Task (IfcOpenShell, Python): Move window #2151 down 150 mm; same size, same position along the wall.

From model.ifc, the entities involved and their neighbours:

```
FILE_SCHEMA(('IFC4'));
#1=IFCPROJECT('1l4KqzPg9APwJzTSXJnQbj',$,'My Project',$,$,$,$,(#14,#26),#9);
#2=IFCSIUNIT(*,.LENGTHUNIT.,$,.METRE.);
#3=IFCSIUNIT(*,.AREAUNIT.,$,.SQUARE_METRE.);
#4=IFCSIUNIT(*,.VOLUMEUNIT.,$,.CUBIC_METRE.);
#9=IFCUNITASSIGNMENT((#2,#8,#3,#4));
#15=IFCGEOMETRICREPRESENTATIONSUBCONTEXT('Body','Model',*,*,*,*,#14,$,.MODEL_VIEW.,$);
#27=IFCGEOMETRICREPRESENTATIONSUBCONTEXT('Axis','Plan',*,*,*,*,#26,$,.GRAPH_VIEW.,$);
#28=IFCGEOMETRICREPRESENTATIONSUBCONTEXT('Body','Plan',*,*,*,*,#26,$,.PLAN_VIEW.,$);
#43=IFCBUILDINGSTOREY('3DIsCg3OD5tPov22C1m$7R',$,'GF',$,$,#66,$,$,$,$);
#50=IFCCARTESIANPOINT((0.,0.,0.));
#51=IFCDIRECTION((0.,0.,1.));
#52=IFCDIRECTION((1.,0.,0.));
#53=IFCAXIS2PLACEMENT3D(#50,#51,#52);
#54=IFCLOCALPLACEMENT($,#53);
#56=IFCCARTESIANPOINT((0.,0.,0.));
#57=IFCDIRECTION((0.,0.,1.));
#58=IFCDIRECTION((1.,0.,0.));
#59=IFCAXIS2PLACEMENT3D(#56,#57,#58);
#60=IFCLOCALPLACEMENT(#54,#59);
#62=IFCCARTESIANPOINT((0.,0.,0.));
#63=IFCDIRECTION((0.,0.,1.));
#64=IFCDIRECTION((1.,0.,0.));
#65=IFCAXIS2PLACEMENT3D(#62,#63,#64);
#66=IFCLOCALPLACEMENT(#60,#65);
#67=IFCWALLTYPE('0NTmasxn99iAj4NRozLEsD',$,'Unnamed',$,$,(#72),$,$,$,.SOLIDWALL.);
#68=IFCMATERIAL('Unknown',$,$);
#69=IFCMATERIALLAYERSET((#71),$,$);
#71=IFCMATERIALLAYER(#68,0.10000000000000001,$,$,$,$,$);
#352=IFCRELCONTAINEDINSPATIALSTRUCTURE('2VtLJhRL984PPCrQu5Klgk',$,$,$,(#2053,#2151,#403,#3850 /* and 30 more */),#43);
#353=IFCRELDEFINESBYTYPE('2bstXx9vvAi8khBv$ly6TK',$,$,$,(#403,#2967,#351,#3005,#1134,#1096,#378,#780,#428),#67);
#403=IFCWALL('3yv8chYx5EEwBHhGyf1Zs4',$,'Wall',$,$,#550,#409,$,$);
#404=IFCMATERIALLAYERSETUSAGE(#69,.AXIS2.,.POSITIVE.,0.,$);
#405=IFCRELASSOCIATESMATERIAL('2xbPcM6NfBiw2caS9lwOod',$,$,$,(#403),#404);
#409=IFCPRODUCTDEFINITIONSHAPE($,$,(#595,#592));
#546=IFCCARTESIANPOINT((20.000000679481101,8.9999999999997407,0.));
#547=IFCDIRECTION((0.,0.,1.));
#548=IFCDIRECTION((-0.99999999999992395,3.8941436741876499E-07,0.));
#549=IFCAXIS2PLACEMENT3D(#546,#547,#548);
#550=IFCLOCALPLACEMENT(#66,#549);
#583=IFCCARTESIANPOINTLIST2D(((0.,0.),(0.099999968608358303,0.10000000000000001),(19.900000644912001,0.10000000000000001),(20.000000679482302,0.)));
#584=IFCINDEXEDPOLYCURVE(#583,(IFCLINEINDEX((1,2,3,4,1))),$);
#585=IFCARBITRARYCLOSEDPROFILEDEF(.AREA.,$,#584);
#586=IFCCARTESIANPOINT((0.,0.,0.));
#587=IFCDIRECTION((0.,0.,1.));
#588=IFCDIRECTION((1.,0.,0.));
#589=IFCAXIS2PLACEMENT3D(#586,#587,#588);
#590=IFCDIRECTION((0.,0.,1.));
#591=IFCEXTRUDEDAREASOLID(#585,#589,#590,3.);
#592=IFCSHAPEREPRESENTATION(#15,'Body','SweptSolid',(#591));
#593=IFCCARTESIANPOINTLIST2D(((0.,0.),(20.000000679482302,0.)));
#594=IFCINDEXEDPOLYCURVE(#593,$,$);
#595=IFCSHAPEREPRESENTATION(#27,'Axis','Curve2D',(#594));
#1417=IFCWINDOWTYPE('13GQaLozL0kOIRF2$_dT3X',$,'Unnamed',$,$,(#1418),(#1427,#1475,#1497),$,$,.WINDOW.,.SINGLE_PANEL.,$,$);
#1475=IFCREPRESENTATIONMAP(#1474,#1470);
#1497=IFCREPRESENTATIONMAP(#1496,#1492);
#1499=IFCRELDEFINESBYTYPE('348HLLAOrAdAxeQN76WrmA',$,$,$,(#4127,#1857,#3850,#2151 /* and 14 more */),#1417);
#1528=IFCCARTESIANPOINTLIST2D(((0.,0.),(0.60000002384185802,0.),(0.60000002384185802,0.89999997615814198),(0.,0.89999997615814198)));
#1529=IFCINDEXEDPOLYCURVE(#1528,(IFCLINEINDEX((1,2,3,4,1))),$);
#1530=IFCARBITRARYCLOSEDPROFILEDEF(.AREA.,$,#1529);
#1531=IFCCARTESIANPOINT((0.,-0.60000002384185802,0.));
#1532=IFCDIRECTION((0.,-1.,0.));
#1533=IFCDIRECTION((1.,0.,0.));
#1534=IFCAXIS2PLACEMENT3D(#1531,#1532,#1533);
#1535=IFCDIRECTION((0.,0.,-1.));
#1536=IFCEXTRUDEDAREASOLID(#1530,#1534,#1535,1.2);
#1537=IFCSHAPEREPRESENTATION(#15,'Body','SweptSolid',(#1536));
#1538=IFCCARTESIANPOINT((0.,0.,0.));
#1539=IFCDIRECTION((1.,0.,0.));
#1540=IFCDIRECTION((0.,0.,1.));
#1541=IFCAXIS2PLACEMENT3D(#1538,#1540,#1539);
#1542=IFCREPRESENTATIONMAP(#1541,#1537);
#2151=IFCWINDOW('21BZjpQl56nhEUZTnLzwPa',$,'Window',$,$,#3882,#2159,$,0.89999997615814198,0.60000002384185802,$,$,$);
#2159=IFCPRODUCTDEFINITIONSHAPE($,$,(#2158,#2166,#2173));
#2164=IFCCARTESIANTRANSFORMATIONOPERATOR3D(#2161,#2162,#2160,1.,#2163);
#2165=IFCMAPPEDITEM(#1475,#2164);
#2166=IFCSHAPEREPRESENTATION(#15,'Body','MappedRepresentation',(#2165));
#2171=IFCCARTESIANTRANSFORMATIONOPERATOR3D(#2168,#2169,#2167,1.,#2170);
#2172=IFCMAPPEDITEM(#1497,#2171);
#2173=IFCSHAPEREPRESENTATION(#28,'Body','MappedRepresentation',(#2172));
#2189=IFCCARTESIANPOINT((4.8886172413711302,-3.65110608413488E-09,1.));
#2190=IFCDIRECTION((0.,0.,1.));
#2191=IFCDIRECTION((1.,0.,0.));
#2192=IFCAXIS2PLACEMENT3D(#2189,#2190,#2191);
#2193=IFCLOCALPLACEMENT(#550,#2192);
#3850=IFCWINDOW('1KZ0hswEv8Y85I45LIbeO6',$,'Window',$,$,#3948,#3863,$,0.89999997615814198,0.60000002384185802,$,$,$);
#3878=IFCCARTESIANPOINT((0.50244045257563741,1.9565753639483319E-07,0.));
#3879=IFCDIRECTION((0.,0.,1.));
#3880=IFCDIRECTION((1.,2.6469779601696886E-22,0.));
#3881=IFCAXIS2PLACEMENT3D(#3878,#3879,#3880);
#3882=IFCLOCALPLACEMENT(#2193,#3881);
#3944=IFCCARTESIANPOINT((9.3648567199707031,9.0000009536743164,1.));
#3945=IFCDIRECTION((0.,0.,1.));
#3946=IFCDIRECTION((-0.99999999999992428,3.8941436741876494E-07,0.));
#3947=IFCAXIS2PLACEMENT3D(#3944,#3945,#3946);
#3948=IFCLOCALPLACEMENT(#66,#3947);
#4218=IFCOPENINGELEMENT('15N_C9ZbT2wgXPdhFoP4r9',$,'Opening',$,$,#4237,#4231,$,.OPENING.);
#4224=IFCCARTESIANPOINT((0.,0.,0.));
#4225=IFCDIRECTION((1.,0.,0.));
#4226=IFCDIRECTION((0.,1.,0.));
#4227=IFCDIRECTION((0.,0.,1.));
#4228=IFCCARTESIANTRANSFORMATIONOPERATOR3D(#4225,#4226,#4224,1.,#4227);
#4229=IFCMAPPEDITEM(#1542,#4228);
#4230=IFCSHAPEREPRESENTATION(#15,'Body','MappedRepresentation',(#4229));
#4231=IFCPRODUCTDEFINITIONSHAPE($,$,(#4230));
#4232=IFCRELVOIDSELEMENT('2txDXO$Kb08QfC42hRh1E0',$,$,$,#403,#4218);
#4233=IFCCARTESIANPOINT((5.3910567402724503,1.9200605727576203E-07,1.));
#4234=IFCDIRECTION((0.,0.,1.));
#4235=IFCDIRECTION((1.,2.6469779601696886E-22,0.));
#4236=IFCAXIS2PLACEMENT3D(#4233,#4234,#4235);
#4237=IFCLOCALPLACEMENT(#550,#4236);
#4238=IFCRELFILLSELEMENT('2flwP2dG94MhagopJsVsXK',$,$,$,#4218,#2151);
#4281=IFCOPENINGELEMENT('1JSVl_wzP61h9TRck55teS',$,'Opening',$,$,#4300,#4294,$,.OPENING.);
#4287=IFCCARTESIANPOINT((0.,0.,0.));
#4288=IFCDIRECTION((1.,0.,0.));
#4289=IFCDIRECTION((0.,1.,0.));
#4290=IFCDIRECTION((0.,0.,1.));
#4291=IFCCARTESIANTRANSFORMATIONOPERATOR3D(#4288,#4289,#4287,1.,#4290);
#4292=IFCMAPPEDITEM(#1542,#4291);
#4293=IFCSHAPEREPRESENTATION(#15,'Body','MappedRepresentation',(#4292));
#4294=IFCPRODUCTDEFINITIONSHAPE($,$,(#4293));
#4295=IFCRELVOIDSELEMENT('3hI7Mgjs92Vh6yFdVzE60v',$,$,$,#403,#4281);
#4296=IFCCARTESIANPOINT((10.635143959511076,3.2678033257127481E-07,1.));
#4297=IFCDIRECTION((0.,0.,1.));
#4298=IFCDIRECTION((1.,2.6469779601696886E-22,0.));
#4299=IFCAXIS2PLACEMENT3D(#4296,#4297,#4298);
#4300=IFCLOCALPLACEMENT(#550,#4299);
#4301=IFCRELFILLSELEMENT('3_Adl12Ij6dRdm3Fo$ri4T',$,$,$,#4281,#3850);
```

```python
import numpy as np
import ifcopenshell
import ifcopenshell.api.geometry
import ifcopenshell.util.placement
import ifcopenshell.util.unit

model = ifcopenshell.open("model.ifc")
unit_scale = ifcopenshell.util.unit.calculate_unit_scale(model)

window = model.by_guid("21BZjpQl56nhEUZTnLzwPa")
opening = window.FillsVoids[0].RelatingOpeningElement
dz = -0.15

shift = np.array([0.0, 0.0, dz])
# The window is not placed relative to its opening, so move both.
for product in (opening, window):
    matrix = ifcopenshell.util.placement.get_local_placement(product.ObjectPlacement)
    matrix[:3, 3] += shift
    ifcopenshell.api.geometry.edit_object_placement(model, product=product, matrix=matrix, is_si=False)

print(f"moved by {dz * unit_scale:+.3f} m")

model.write("model_updated.ifc")
```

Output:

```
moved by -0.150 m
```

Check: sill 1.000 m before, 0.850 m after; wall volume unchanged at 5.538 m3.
